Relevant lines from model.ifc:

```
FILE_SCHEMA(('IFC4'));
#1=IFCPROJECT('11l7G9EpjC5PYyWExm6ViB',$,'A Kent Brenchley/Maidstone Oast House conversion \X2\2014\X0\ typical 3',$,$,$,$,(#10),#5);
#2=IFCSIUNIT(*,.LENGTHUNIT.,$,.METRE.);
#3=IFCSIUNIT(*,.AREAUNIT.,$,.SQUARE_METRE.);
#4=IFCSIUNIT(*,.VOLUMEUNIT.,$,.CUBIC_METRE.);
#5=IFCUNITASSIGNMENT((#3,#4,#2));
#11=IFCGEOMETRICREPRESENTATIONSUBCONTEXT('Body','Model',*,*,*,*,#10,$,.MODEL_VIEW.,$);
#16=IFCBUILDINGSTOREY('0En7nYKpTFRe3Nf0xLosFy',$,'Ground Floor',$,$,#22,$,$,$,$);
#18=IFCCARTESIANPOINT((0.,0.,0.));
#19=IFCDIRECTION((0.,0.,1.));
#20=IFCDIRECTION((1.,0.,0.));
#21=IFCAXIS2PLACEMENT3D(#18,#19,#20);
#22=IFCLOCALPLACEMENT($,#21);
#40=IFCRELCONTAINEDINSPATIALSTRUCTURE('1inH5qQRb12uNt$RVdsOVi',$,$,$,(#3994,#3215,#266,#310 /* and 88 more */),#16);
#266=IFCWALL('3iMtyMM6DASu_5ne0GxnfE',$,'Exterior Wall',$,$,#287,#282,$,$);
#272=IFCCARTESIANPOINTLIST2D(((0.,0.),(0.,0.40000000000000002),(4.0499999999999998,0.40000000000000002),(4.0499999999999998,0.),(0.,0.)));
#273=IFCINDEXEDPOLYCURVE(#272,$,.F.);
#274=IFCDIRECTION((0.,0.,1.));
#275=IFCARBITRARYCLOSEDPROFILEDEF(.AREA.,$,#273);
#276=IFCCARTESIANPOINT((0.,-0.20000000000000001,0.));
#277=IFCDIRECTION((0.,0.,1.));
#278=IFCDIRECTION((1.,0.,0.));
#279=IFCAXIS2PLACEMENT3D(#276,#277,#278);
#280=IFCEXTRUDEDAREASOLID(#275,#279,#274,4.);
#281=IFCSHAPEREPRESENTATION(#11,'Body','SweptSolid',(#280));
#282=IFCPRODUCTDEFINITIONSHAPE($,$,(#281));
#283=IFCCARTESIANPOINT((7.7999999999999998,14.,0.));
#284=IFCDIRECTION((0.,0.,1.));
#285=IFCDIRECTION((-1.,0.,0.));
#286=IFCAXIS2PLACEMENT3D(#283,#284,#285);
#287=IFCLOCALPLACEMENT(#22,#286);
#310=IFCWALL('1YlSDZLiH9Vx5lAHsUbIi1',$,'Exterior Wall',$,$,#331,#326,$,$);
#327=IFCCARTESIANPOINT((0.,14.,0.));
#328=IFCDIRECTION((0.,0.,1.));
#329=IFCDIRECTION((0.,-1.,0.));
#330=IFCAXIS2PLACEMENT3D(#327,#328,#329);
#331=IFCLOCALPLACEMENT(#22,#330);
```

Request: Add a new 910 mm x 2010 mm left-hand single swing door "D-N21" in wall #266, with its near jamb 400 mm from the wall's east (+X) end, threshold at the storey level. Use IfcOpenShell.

```python
import numpy as np
import ifcopenshell
import ifcopenshell.api.feature
import ifcopenshell.api.geometry
import ifcopenshell.api.root
import ifcopenshell.api.spatial
import ifcopenshell.geom
import ifcopenshell.util.element
import ifcopenshell.util.placement
import ifcopenshell.util.representation
import ifcopenshell.util.shape
import ifcopenshell.util.unit

model = ifcopenshell.open("model.ifc")
unit_scale = ifcopenshell.util.unit.calculate_unit_scale(model)
settings = ifcopenshell.geom.settings()


def volume(element):
    """Net volume in cubic metres, openings subtracted."""
    shape = ifcopenshell.geom.create_shape(settings, element)
    return ifcopenshell.util.shape.get_volume(shape.geometry)


wall = model.by_id(266)
storey = ifcopenshell.util.element.get_container(wall, ifc_class="IfcBuildingStorey")
context = ifcopenshell.util.representation.get_context(model, "Model", "Body", "MODEL_VIEW")
before = volume(wall)

width, height, from_end, sill = 0.91, 2.01, 0.4, 0.0  # metres

# The wall runs along its own X axis, and the end named is its -X end.
wall_shape = ifcopenshell.geom.create_shape(settings, wall)
x, y, z = ifcopenshell.util.shape.get_vertices(wall_shape.geometry).T
start = x.min() + from_end
face, thickness = float(y.min()), float(y.max() - y.min())
wall_matrix = ifcopenshell.util.placement.get_local_placement(wall.ObjectPlacement)
level = ifcopenshell.util.placement.get_local_placement(storey.ObjectPlacement)[2, 3]


def in_wall(x, y):
    """Placement at x, y metres in the wall's axes, at sill height."""
    matrix = wall_matrix.copy()
    matrix[:, 3] = wall_matrix @ np.array([x / unit_scale, y / unit_scale, 0.0, 1.0])
    matrix[2, 3] = level + sill / unit_scale
    return matrix


# Opening: a box that overshoots both wall faces by 50 mm.
opening = ifcopenshell.api.root.create_entity(model, ifc_class="IfcOpeningElement", predefined_type="OPENING")
box = ifcopenshell.api.geometry.add_wall_representation(
    model, context=context, length=width, height=height, thickness=thickness + 0.1
)
ifcopenshell.api.geometry.assign_representation(model, product=opening, representation=box)
ifcopenshell.api.geometry.edit_object_placement(model, product=opening, matrix=in_wall(start, face - 0.05), is_si=False)
ifcopenshell.api.feature.add_feature(model, feature=opening, element=wall)

door = ifcopenshell.api.root.create_entity(model, ifc_class="IfcDoor", name="D-N21", predefined_type="DOOR")
door.OverallWidth, door.OverallHeight = width / unit_scale, height / unit_scale
door.OperationType = "SINGLE_SWING_LEFT"
body = ifcopenshell.api.geometry.add_door_representation(
    model,
    context=context,
    overall_width=door.OverallWidth,
    overall_height=door.OverallHeight,
    operation_type="SINGLE_SWING_LEFT",
    lining_properties={"LiningDepth": thickness / unit_scale, "ThresholdDepth": thickness / unit_scale},
)
ifcopenshell.api.geometry.assign_representation(model, product=door, representation=body)
ifcopenshell.api.spatial.assign_container(model, products=[door], relating_structure=storey)
ifcopenshell.api.feature.add_filling(model, opening=opening, element=door)

# The lining spans the wall, so the door starts at the wall face.
ifcopenshell.api.geometry.edit_object_placement(model, product=door, matrix=in_wall(start, face), is_si=False)

after = volume(wall)

print(f"wall volume {before:.3f} -> {after:.3f} m3")

model.write("model-out.ifc")
```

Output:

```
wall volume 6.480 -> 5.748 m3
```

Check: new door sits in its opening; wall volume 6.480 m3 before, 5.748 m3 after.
